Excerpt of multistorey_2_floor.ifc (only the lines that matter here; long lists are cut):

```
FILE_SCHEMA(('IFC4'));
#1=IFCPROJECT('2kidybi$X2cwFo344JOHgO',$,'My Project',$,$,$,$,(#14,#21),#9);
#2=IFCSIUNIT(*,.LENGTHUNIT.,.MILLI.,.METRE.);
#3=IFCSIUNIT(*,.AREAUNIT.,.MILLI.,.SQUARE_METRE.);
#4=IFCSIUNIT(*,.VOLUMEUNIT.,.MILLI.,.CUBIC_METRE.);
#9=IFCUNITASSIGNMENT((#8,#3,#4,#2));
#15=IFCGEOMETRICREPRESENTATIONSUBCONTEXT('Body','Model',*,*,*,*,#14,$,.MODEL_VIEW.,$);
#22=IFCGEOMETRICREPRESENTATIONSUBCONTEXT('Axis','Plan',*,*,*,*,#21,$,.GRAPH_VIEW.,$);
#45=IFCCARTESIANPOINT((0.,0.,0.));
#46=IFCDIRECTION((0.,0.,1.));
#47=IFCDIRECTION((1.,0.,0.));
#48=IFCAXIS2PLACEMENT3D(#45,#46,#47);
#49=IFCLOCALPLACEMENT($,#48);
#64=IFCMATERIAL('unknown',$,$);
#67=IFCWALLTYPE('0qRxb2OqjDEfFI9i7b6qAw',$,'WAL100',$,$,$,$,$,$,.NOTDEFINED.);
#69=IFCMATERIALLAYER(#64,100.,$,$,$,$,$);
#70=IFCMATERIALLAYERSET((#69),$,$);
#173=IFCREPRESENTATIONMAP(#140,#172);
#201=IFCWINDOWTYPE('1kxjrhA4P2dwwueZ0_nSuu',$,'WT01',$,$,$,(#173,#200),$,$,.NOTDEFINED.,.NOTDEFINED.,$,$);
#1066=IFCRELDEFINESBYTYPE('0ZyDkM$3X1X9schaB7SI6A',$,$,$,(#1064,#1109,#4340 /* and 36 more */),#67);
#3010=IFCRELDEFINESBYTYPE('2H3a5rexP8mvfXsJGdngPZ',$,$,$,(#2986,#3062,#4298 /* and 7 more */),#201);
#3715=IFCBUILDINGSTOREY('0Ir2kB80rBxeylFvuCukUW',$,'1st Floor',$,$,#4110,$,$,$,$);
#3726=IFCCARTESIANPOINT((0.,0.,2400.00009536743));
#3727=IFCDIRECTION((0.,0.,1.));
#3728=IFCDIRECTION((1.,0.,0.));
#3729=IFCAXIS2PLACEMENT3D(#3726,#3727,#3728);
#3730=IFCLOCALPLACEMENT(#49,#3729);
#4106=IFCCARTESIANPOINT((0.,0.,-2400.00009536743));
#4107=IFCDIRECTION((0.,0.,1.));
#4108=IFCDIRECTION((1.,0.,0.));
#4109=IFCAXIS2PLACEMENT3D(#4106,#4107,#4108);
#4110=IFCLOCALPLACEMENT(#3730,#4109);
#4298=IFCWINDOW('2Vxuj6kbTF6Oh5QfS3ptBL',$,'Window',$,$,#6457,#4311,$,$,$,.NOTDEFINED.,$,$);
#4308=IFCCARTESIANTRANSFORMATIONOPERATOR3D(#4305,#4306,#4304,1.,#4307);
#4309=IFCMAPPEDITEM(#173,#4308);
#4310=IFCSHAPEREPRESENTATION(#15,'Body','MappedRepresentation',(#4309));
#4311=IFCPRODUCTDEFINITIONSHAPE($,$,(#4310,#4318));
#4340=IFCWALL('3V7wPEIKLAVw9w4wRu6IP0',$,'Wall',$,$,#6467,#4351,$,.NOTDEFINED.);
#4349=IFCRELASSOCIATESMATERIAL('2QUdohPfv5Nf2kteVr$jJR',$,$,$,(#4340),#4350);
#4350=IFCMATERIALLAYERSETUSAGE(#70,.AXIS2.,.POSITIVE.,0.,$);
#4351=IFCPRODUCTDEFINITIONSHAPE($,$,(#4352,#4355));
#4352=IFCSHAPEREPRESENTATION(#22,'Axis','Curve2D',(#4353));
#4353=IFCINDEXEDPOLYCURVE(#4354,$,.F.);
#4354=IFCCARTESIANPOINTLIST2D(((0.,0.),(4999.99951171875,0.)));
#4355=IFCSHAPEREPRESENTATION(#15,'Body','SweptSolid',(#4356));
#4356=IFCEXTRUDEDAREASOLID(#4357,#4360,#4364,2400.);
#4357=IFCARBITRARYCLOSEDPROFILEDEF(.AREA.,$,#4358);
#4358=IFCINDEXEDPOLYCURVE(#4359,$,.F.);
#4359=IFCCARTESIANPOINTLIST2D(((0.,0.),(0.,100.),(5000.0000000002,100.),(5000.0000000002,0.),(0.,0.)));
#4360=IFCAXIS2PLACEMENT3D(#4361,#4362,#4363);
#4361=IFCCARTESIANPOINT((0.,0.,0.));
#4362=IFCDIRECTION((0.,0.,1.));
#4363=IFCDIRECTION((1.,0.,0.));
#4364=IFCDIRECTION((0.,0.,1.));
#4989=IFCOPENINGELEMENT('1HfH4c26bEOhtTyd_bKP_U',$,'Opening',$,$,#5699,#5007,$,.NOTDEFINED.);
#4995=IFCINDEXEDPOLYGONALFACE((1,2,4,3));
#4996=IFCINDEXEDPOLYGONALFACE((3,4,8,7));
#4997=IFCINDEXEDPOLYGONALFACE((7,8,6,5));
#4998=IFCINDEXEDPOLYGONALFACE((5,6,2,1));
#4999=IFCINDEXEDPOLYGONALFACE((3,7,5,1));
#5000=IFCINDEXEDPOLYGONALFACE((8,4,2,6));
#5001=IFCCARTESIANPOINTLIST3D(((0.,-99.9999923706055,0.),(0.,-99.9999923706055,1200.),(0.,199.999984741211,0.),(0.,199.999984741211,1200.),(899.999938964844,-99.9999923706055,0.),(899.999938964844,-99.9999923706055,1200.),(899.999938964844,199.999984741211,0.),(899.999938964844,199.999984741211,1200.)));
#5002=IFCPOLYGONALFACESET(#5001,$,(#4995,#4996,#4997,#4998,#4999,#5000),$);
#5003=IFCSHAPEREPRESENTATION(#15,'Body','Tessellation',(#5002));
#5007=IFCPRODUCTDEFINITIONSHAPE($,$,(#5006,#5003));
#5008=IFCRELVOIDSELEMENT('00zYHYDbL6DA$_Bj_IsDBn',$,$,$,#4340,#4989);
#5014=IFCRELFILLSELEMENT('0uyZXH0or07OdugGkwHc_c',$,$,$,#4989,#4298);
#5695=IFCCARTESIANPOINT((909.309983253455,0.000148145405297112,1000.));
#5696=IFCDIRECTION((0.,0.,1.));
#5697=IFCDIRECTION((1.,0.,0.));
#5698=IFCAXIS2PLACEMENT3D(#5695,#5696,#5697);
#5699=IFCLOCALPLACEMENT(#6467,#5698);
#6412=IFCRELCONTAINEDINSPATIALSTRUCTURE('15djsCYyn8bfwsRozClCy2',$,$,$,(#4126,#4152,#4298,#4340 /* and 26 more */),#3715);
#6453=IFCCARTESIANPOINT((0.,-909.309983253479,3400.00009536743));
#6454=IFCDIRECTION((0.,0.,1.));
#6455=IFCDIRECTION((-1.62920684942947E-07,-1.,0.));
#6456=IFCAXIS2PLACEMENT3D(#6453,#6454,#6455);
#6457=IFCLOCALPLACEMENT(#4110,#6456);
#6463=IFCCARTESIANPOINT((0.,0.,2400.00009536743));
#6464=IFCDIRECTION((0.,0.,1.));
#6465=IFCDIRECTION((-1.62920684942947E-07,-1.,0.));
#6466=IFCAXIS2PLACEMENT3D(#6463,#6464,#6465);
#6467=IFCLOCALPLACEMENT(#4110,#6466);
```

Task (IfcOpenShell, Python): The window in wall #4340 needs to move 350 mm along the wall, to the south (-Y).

```python
import ifcopenshell
import ifcopenshell.api.geometry
import ifcopenshell.util.placement

model = ifcopenshell.open("multistorey_2_floor.ifc")

window = model.by_guid("2Vxuj6kbTF6Oh5QfS3ptBL")
opening = window.FillsVoids[0].RelatingOpeningElement
wall = opening.VoidsElements[0].RelatingBuildingElement

wall_matrix = ifcopenshell.util.placement.get_local_placement(wall.ObjectPlacement)
shift = wall_matrix[:3, 0] * 350.0
before = ifcopenshell.util.placement.get_local_placement(window.ObjectPlacement)[:3, 3].copy()

# The window is not placed relative to its opening, so move both.
for product in (opening, window):
    matrix = ifcopenshell.util.placement.get_local_placement(product.ObjectPlacement)
    matrix[:3, 3] += shift
    ifcopenshell.api.geometry.edit_object_placement(model, product=product, matrix=matrix, is_si=False)

after = ifcopenshell.util.placement.get_local_placement(window.ObjectPlacement)[:3, 3]
print("window moved by", (after - before).round(3) + 0.0)

model.write("multistorey_2_floor_updated.ifc")
```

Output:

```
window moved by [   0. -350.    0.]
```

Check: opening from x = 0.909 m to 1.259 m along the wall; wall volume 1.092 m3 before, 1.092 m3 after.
